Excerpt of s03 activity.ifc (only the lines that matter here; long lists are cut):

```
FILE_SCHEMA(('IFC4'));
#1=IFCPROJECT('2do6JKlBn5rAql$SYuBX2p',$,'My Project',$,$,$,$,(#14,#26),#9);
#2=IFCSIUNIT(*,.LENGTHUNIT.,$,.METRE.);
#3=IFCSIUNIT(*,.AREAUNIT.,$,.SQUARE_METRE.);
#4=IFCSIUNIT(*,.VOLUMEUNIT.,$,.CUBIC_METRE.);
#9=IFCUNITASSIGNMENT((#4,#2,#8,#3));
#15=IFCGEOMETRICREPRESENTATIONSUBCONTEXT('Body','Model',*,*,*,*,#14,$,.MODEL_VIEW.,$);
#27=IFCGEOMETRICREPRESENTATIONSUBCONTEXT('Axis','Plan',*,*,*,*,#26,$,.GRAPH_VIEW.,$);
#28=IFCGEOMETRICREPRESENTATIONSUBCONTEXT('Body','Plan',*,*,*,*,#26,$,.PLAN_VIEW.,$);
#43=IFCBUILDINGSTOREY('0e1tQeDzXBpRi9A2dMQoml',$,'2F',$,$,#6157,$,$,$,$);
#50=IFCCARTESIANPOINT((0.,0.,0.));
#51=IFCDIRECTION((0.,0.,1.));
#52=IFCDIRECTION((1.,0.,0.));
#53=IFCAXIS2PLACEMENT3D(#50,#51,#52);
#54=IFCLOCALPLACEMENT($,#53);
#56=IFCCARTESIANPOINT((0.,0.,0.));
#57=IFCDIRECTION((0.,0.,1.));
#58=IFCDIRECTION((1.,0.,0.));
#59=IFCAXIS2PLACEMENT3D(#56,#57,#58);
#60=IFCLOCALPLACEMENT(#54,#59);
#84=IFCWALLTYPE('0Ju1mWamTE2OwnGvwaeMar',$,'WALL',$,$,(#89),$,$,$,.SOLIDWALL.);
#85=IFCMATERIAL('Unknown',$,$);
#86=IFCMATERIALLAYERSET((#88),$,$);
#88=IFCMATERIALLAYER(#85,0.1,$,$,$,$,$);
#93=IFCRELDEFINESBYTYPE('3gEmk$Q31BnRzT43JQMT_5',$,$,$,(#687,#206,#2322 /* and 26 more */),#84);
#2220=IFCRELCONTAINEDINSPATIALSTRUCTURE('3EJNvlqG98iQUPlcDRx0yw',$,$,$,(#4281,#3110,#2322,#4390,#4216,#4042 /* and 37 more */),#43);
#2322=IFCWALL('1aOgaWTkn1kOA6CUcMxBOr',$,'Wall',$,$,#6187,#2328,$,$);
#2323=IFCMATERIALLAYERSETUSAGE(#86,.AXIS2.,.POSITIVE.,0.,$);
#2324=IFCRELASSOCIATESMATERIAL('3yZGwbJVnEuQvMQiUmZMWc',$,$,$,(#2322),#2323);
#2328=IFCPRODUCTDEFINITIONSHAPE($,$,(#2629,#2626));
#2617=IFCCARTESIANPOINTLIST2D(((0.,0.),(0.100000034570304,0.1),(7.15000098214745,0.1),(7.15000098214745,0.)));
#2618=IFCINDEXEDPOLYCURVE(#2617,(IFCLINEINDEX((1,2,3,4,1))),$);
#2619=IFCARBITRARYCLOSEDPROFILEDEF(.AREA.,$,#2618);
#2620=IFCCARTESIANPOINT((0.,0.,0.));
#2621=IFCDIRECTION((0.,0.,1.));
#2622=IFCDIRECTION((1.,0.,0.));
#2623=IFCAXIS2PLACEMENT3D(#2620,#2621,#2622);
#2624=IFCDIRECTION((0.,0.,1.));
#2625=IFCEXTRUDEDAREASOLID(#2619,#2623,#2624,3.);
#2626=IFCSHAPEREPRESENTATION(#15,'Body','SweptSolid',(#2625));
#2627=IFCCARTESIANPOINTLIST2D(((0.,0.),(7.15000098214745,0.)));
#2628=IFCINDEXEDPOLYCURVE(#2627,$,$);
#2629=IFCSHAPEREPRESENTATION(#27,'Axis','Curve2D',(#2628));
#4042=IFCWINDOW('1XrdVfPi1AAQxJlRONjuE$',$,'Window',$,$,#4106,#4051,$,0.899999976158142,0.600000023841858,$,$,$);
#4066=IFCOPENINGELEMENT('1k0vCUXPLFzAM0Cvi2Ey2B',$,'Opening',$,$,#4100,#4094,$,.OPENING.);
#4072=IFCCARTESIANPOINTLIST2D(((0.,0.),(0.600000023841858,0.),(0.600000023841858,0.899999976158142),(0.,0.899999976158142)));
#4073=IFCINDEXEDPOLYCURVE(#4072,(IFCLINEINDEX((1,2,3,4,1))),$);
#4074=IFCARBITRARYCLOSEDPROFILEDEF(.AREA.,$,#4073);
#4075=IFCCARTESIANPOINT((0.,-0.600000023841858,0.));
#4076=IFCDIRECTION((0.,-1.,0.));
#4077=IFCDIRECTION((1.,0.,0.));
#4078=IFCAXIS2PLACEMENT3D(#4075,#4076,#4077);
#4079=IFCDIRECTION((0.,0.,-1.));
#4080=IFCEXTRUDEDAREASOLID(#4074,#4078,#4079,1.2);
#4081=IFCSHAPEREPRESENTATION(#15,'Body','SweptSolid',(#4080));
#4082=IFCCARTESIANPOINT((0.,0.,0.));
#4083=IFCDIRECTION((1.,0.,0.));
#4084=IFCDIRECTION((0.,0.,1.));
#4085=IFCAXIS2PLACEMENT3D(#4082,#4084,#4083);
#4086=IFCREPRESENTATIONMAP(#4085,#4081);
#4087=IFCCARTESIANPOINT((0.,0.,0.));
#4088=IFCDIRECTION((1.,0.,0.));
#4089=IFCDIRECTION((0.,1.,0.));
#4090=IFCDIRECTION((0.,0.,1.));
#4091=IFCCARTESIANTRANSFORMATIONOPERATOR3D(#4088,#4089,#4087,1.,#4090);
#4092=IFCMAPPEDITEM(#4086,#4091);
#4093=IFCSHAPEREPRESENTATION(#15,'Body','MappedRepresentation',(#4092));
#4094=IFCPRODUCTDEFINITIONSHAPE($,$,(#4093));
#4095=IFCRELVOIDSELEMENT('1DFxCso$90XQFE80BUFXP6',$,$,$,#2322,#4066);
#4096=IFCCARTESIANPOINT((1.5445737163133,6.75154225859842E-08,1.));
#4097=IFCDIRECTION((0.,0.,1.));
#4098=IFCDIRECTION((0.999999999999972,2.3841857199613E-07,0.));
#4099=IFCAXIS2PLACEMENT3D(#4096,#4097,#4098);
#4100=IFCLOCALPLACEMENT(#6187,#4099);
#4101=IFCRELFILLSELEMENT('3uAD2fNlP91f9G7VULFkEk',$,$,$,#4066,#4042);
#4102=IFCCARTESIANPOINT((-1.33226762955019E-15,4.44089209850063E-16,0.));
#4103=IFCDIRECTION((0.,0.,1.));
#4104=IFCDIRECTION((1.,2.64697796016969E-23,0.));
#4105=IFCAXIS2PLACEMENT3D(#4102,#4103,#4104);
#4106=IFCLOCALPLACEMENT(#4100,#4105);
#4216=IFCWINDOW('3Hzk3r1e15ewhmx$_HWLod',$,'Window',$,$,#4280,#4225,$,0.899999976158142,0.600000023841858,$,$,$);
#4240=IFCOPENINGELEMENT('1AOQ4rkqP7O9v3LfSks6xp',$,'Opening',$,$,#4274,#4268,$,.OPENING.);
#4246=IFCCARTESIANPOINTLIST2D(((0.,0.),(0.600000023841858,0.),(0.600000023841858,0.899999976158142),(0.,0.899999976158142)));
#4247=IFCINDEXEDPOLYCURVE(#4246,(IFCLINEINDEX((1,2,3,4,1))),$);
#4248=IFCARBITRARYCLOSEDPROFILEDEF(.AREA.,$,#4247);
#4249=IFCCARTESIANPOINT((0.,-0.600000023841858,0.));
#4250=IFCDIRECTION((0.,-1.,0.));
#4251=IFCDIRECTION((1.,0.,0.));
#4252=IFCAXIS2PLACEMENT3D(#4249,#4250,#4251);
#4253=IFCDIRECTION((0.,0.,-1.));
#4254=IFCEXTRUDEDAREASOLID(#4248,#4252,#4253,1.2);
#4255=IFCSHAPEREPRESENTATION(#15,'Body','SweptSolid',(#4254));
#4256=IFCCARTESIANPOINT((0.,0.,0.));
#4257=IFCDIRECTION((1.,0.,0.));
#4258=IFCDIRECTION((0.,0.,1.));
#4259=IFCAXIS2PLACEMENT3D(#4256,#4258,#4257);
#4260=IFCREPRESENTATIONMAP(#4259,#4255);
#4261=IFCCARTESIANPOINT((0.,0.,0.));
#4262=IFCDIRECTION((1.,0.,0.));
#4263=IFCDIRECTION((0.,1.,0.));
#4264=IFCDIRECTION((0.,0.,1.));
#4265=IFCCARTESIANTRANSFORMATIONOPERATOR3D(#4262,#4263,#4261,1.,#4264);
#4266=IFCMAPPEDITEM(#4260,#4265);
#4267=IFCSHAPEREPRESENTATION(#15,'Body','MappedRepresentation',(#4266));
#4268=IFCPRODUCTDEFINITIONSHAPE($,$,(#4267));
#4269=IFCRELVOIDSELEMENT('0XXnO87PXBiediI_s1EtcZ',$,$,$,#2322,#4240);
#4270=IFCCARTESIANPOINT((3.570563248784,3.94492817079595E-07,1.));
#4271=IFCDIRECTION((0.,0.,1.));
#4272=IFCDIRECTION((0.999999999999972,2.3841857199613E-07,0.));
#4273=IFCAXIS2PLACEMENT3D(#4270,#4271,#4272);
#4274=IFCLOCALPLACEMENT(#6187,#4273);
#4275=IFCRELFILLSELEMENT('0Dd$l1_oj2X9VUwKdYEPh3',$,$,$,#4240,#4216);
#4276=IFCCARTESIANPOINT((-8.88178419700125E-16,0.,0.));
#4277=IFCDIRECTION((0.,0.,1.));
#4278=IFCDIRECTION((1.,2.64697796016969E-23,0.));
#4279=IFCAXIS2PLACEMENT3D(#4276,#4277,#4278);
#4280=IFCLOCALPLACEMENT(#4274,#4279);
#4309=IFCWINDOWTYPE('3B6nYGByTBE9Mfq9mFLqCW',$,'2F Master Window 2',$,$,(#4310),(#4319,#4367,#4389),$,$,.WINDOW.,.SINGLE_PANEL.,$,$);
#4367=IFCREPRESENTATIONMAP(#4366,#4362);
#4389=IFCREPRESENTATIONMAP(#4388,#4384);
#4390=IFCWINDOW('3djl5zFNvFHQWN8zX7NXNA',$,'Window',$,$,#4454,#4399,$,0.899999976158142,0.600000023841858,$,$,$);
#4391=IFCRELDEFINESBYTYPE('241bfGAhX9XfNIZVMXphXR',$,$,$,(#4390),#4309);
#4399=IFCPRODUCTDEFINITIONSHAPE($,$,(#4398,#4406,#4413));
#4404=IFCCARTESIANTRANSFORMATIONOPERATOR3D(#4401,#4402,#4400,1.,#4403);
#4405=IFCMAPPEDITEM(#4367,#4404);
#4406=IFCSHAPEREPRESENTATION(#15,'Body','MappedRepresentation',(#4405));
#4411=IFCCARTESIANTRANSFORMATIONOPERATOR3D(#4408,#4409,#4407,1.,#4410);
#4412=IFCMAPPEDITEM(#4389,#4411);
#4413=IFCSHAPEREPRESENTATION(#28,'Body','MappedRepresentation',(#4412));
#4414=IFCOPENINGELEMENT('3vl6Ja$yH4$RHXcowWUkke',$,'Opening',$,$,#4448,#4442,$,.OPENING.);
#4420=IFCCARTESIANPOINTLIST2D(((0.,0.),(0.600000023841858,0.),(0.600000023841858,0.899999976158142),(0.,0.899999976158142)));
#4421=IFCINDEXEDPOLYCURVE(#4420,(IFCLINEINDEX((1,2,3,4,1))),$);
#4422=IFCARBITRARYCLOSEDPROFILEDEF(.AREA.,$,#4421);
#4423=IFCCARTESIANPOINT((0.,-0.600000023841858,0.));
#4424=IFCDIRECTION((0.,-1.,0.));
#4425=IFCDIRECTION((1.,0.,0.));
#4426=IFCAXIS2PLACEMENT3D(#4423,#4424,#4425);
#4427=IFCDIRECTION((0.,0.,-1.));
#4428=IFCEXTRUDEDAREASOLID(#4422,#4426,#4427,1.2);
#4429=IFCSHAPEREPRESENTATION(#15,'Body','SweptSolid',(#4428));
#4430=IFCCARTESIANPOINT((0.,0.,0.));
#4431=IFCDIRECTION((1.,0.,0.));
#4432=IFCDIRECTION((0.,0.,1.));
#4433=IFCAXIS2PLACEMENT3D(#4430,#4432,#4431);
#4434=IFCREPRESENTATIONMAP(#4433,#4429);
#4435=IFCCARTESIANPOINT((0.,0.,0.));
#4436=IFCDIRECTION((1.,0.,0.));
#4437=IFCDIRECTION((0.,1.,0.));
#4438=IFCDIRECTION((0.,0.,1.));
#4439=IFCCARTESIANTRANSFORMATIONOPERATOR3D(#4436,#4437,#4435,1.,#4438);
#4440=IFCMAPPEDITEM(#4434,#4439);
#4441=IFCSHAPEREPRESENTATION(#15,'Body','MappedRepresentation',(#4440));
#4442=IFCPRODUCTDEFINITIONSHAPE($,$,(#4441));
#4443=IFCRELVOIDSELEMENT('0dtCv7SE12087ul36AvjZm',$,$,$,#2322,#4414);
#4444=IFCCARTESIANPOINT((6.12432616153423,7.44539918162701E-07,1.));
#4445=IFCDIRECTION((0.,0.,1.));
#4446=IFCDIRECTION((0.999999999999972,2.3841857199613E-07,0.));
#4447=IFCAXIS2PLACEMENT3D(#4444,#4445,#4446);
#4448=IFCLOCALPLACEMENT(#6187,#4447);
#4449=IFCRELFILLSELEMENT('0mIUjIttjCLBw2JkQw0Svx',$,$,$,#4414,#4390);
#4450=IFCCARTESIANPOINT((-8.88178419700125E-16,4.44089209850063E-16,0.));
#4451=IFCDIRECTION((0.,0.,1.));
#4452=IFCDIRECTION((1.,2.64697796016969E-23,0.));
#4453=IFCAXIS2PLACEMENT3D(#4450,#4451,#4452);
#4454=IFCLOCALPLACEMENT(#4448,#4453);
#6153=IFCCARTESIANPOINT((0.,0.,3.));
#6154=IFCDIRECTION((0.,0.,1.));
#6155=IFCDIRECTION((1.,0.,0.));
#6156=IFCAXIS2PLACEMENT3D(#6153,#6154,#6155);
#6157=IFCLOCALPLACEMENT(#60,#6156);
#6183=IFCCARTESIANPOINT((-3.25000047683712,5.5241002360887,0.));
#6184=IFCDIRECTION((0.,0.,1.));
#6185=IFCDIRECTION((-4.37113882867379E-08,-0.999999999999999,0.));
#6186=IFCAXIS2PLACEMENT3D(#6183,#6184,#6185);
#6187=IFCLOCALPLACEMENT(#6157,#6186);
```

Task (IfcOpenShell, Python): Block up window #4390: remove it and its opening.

```python
import ifcopenshell
import ifcopenshell.api.feature
import ifcopenshell.api.root
import ifcopenshell.geom
import ifcopenshell.util.shape

model = ifcopenshell.open("s03 activity.ifc")
settings = ifcopenshell.geom.settings()


def volume(element):
    """Net volume in cubic metres, openings subtracted."""
    shape = ifcopenshell.geom.create_shape(settings, element)
    return ifcopenshell.util.shape.get_volume(shape.geometry)


window = model.by_guid("3djl5zFNvFHQWN8zX7NXNA")
opening = window.FillsVoids[0].RelatingOpeningElement
wall = opening.VoidsElements[0].RelatingBuildingElement
before = volume(wall)

ifcopenshell.api.root.remove_product(model, product=window)
ifcopenshell.api.feature.remove_feature(model, feature=opening)

after = volume(wall)

print(f"wall volume {before:.3f} -> {after:.3f} m3")

model.write("s03 activity_updated.ifc")
```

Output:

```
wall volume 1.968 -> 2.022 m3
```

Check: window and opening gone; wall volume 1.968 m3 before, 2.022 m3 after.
